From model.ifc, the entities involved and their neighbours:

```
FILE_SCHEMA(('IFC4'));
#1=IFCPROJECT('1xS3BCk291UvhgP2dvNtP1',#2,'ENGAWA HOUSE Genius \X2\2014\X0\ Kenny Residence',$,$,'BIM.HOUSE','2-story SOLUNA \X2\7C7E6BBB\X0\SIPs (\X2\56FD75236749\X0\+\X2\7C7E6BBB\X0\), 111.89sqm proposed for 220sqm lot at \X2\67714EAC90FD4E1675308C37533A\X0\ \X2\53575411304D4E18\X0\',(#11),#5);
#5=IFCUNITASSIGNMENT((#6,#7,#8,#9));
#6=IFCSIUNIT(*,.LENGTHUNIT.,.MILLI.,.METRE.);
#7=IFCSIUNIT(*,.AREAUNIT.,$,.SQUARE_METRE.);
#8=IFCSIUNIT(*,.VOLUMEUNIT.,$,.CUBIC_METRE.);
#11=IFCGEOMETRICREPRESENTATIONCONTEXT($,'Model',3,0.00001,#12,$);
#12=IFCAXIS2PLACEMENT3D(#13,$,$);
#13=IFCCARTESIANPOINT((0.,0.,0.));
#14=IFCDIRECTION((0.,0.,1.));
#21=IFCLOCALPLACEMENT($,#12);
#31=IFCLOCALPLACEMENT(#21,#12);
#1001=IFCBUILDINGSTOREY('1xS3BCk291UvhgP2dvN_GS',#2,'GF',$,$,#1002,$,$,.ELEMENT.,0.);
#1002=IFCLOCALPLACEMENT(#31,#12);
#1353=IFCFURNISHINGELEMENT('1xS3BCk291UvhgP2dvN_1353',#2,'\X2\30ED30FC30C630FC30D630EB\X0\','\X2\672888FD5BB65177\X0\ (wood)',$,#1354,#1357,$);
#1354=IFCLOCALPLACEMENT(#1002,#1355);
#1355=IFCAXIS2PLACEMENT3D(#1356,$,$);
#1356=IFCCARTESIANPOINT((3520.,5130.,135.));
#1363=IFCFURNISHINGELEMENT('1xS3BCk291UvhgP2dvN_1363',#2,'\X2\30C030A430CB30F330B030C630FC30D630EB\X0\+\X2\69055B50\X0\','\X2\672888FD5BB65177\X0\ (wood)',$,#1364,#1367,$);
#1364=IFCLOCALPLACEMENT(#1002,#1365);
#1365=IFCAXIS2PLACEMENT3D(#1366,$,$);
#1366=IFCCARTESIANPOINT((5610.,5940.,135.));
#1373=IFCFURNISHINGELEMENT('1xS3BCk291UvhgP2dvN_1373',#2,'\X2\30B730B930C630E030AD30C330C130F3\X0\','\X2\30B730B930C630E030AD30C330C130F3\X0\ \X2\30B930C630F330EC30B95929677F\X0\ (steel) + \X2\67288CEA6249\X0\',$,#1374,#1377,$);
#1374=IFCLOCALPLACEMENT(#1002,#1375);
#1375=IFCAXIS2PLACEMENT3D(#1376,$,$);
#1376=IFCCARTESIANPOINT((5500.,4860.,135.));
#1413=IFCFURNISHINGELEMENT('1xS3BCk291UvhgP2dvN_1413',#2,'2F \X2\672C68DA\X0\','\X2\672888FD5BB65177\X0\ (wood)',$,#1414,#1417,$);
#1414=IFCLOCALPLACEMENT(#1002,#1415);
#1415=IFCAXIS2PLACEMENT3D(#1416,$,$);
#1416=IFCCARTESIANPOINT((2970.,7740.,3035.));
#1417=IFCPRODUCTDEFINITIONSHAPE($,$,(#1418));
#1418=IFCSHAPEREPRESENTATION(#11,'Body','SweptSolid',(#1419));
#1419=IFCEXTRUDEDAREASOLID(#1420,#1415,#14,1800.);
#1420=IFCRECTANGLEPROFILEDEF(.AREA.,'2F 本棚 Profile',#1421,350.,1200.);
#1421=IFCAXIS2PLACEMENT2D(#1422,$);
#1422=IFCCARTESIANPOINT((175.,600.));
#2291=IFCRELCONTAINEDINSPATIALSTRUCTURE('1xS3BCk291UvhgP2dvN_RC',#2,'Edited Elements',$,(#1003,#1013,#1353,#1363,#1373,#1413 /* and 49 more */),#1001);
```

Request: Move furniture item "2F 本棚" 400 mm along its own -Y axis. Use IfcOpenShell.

```python
import ifcopenshell
import ifcopenshell.api.geometry
import ifcopenshell.util.placement

model = ifcopenshell.open("model.ifc")

item = model.by_guid("1xS3BCk291UvhgP2dvN_1413")
matrix = ifcopenshell.util.placement.get_local_placement(item.ObjectPlacement)
matrix[:3, 3] -= matrix[:3, 1] * 400.0
ifcopenshell.api.geometry.edit_object_placement(model, product=item, matrix=matrix, is_si=False)

print(ifcopenshell.util.placement.get_local_placement(item.ObjectPlacement).round(3) + 0.0)

model.write("model_rev.ifc")
```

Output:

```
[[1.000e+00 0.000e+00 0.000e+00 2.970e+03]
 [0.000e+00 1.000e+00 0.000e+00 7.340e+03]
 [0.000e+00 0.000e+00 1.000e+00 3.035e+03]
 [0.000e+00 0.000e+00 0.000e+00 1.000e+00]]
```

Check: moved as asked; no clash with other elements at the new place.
